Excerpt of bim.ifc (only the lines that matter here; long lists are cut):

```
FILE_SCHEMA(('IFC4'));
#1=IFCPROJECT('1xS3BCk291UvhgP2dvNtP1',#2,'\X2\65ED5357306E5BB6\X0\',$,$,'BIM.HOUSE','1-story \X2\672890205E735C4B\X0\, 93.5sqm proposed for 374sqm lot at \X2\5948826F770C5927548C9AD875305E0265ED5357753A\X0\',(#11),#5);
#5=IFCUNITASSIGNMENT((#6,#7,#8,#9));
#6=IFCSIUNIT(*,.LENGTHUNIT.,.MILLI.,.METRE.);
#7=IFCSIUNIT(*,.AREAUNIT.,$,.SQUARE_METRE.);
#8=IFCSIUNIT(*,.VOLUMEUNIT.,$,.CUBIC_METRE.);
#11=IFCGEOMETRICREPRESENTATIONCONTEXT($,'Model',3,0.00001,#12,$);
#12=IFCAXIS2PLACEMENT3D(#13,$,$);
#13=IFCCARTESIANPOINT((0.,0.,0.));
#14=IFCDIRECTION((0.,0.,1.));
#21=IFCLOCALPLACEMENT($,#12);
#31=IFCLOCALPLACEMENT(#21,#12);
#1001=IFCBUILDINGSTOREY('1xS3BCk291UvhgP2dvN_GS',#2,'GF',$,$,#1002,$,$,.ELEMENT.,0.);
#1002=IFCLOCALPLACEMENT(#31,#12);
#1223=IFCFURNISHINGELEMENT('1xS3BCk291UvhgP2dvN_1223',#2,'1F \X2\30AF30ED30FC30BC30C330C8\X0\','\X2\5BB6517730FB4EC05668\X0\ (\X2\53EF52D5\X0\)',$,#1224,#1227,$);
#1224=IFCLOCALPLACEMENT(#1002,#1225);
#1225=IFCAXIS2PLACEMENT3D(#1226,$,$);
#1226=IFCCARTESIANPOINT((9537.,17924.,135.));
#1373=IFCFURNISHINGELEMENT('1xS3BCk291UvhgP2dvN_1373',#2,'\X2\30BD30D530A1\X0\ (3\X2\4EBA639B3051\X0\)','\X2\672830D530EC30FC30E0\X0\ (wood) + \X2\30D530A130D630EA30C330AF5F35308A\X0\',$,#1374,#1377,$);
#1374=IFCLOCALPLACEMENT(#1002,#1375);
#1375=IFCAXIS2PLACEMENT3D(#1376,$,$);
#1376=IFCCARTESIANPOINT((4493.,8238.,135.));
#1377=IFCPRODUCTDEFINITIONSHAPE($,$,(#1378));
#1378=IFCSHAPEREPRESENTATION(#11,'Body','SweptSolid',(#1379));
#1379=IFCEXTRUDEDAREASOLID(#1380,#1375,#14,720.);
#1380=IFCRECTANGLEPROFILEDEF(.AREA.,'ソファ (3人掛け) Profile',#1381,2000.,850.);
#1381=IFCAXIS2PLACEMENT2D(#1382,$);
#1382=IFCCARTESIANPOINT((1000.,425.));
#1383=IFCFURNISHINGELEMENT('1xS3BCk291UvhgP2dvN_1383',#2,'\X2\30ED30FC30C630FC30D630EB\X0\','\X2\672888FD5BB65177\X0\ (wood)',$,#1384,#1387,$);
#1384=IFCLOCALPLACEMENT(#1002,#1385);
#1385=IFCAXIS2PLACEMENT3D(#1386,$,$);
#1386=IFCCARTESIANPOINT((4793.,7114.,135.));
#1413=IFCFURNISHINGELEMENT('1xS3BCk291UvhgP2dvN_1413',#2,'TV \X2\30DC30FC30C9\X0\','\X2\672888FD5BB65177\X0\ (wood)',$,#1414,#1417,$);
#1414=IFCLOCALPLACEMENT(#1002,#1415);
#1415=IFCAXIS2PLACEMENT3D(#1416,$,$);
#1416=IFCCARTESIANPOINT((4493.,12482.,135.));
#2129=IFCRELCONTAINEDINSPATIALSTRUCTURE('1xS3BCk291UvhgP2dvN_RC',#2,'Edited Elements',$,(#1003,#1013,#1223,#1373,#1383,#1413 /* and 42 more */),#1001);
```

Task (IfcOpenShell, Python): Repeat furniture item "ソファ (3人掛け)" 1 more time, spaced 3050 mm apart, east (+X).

```python
import numpy as np
import ifcopenshell
import ifcopenshell.api.geometry
import ifcopenshell.api.root
import ifcopenshell.util.element
import ifcopenshell.util.placement

model = ifcopenshell.open("bim.ifc")


def reuse_history(source, copy):
    """copy_class also copies each property set's owner history, people and application; keep the originals."""
    for rel in copy.IsDefinedBy:
        if rel.is_a("IfcRelDefinesByProperties") and (history := rel.RelatingPropertyDefinition.OwnerHistory):
            rel.RelatingPropertyDefinition.OwnerHistory = source.OwnerHistory
            ifcopenshell.util.element.remove_deep2(model, history)


source = model.by_id(1373)
base = ifcopenshell.util.placement.get_local_placement(source.ObjectPlacement)
step = np.array([1.0, 0.0, 0.0]) * 3050.0

for i in range(1, 2):
    copy = ifcopenshell.api.root.copy_class(model, product=source)
    copy.Representation = ifcopenshell.util.element.copy_deep(
        model, source.Representation, exclude=["IfcGeometricRepresentationContext", "IfcRepresentationMap"]
    )
    reuse_history(source, copy)
    matrix = base.copy()
    matrix[:3, 3] += i * step
    print("added at", matrix[:3, 3].round(3) + 0.0)
    ifcopenshell.api.geometry.edit_object_placement(model, product=copy, matrix=matrix, is_si=False)

model.write("bim_v2.ifc")
```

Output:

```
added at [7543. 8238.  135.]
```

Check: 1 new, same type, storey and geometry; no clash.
